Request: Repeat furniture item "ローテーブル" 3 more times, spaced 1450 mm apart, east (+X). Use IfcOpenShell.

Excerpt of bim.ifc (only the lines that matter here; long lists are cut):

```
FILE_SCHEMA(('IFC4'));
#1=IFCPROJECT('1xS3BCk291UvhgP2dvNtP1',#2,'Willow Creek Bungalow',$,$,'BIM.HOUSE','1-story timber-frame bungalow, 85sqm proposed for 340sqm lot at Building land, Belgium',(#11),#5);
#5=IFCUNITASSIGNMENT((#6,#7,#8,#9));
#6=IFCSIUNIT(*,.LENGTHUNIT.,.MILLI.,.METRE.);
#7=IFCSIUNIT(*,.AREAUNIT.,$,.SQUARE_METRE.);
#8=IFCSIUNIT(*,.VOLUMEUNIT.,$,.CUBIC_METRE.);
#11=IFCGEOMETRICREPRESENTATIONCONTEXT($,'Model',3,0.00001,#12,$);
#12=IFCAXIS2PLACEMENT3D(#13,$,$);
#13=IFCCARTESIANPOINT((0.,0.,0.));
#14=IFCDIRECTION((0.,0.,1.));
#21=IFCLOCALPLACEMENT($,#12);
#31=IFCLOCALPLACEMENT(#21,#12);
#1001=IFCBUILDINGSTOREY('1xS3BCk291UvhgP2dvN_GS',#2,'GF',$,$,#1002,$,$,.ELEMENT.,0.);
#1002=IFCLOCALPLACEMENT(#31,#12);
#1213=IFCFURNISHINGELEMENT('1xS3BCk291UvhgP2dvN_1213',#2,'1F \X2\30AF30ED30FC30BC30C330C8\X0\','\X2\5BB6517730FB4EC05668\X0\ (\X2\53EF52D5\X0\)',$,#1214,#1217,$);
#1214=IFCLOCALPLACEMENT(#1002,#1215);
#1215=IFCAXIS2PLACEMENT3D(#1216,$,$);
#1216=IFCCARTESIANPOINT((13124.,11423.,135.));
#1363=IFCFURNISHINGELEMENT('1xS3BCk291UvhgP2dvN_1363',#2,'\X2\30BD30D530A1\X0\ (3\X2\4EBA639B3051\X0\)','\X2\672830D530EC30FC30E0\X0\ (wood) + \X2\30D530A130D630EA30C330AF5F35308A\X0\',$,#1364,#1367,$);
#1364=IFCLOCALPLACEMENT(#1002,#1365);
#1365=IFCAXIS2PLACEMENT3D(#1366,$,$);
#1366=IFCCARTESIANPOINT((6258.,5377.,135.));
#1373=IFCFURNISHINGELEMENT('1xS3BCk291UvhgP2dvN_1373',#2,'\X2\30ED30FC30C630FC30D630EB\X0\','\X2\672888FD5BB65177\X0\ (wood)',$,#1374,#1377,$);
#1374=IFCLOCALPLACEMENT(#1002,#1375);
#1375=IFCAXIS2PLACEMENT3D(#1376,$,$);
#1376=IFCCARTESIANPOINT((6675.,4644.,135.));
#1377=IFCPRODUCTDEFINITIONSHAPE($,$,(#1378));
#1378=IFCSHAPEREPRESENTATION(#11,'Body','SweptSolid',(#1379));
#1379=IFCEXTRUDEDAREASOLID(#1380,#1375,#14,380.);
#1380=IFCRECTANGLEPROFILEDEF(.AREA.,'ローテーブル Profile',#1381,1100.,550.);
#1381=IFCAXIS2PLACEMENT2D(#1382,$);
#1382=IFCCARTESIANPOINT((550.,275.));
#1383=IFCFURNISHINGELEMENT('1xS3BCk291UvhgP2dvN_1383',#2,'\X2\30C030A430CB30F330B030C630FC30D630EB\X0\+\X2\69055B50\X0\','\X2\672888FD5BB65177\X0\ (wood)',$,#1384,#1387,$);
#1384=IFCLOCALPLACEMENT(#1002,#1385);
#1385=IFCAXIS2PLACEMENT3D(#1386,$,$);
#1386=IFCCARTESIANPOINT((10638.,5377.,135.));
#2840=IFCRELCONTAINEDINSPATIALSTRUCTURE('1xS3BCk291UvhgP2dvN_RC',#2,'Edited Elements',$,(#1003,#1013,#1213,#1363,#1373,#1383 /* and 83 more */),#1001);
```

```python
import numpy as np
import ifcopenshell
import ifcopenshell.api.geometry
import ifcopenshell.api.root
import ifcopenshell.util.element
import ifcopenshell.util.placement
import ifcopenshell.util.unit

model = ifcopenshell.open("bim.ifc")
unit_scale = ifcopenshell.util.unit.calculate_unit_scale(model)


def reuse_history(source, copy):
    """copy_class also copies each property set's owner history, people and application; keep the originals."""
    for rel in copy.IsDefinedBy:
        if rel.is_a("IfcRelDefinesByProperties") and (history := rel.RelatingPropertyDefinition.OwnerHistory):
            rel.RelatingPropertyDefinition.OwnerHistory = source.OwnerHistory
            ifcopenshell.util.element.remove_deep2(model, history)


source = model.by_guid("1xS3BCk291UvhgP2dvN_1373")
base = ifcopenshell.util.placement.get_local_placement(source.ObjectPlacement)
step = np.array([1.0, 0.0, 0.0]) * 1.45 / unit_scale

for i in range(1, 4):
    copy = ifcopenshell.api.root.copy_class(model, product=source)
    copy.Representation = ifcopenshell.util.element.copy_deep(
        model, source.Representation, exclude=["IfcGeometricRepresentationContext", "IfcRepresentationMap"]
    )
    reuse_history(source, copy)
    matrix = base.copy()
    matrix[:3, 3] += i * step
    print("added at", matrix[:3, 3].round(3) + 0.0)
    ifcopenshell.api.geometry.edit_object_placement(model, product=copy, matrix=matrix, is_si=False)

model.write("bim_edited.ifc")
```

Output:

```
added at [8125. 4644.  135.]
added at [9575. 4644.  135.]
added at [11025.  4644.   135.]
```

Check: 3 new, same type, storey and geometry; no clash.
